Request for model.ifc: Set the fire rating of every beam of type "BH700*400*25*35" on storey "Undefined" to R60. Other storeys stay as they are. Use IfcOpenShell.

First a look at what the model holds.

```python
import ifcopenshell
import ifcopenshell.util.element

model = ifcopenshell.open("model.ifc")
print(model.schema)
storey = next(s for s in model.by_type("IfcBuildingStorey") if s.Name == "Undefined")
beams = [e for e in ifcopenshell.util.element.get_decomposition(storey) if e.is_a("IfcBeam")]
seen = {}
for e in beams:
    element_type = ifcopenshell.util.element.get_type(e)
    key = (element_type.Name if element_type != e and element_type else None, ifcopenshell.util.element.get_pset(e, "Pset_BeamCommon", "FireRating"))
    seen[key] = seen.get(key, 0) + 1
for (name, value), count in sorted(seen.items(), key=str):
    print(count, "x", name, "|", value)
```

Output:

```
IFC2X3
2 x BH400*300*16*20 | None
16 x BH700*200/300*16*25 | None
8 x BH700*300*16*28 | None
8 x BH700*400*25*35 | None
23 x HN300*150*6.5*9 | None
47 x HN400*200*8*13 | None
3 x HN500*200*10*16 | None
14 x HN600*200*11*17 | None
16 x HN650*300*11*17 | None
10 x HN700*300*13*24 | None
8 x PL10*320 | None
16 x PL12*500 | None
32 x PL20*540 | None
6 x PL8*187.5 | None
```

```python
import ifcopenshell
import ifcopenshell.api.pset
import ifcopenshell.util.element

model = ifcopenshell.open("model.ifc")

storey = next(s for s in model.by_type("IfcBuildingStorey") if s.Name == "Undefined")
beams = [e for e in ifcopenshell.util.element.get_decomposition(storey) if e.is_a("IfcBeam")]

count = 0
for e in beams:
    element_type = ifcopenshell.util.element.get_type(e)
    if element_type in (None, e) or element_type.Name != "BH700*400*25*35":
        continue
    # add_pset returns the element's existing set when there is one.
    pset = ifcopenshell.api.pset.add_pset(model, product=e, name="Pset_BeamCommon")
    ifcopenshell.api.pset.edit_pset(model, pset=pset, properties={"FireRating": "R60"})
    count += 1

print(count, "beams updated")

model.write("model_rev.ifc")
```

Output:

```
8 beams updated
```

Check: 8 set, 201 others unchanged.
